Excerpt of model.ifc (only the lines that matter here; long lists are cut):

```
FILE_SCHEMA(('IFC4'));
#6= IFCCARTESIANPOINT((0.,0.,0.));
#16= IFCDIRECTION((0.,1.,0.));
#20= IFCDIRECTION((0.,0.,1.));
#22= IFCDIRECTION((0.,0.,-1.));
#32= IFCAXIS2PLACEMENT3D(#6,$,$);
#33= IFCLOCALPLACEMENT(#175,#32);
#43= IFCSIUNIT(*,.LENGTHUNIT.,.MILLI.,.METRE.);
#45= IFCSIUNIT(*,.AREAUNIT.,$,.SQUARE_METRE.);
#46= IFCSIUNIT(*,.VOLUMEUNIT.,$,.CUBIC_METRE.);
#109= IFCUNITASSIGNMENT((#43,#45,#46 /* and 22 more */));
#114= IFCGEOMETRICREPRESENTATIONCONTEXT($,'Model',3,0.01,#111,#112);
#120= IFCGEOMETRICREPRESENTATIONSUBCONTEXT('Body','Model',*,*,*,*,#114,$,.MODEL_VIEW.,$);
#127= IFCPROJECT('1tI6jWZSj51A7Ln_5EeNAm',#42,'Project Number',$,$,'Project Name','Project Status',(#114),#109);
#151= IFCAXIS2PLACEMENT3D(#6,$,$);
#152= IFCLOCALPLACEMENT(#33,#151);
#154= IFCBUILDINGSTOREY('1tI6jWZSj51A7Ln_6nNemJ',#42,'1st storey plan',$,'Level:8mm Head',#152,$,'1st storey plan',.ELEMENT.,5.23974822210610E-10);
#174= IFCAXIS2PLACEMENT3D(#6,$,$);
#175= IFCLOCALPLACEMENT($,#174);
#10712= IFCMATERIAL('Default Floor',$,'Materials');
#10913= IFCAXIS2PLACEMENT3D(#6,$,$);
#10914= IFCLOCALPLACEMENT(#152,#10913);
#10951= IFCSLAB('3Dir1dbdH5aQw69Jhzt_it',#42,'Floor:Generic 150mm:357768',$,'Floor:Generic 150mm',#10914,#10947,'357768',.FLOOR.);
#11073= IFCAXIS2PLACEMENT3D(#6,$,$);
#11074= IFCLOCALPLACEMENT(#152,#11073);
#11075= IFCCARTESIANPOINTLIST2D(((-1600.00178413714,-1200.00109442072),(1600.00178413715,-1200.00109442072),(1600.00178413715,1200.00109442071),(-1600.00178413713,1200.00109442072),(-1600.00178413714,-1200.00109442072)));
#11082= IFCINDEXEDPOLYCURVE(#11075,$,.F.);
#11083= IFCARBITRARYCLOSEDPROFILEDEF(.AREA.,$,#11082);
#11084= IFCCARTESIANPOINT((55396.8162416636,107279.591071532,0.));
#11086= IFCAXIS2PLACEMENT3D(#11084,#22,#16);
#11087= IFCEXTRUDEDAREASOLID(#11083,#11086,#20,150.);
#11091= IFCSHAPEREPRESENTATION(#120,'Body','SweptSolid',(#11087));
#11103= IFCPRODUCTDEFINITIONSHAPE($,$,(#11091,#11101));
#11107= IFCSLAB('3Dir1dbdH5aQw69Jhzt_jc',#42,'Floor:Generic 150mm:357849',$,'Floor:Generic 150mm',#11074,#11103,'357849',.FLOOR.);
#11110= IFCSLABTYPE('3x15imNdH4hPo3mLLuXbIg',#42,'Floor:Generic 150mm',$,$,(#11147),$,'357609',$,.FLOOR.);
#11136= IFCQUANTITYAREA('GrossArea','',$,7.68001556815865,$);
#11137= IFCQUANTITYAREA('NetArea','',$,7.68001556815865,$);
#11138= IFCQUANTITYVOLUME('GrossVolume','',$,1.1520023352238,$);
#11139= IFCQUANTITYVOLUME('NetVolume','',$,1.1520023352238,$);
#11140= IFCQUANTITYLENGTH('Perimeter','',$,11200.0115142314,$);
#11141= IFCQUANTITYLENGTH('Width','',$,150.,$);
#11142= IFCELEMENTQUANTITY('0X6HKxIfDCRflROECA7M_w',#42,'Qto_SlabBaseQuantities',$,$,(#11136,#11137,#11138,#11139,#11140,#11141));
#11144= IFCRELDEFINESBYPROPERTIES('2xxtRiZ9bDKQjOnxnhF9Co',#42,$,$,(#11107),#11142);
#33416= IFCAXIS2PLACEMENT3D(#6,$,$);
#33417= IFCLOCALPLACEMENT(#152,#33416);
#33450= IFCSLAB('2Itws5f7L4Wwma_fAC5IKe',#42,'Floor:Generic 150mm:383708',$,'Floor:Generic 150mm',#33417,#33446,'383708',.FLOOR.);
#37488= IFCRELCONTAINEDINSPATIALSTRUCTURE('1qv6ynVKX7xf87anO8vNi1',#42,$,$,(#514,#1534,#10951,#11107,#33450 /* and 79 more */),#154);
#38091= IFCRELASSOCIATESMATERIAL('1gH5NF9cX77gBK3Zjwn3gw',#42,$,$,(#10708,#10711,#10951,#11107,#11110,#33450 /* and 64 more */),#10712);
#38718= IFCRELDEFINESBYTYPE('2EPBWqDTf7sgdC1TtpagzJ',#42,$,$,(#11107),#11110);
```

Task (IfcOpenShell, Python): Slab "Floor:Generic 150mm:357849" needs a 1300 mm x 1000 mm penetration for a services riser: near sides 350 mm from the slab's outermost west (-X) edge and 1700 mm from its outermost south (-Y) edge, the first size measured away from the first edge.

```python
import numpy as np
import ifcopenshell
import ifcopenshell.api.feature
import ifcopenshell.api.geometry
import ifcopenshell.api.pset
import ifcopenshell.api.root
import ifcopenshell.geom
import ifcopenshell.util.element
import ifcopenshell.util.placement
import ifcopenshell.util.representation
import ifcopenshell.util.shape
import ifcopenshell.util.unit

model = ifcopenshell.open("model.ifc")
unit_scale = ifcopenshell.util.unit.calculate_unit_scale(model)
area_scale = ifcopenshell.util.unit.calculate_unit_scale(model, "AREAUNIT")
volume_scale = ifcopenshell.util.unit.calculate_unit_scale(model, "VOLUMEUNIT")
settings = ifcopenshell.geom.settings()


def volume(element):
    """Net volume in cubic metres, openings subtracted."""
    shape = ifcopenshell.geom.create_shape(settings, element)
    return ifcopenshell.util.shape.get_volume(shape.geometry)


slab = model.by_guid("3Dir1dbdH5aQw69Jhzt_jc")
before = volume(slab)

# Extent in the slab's own axes, in metres. The edges named are its -X and -Y sides.
slab_shape = ifcopenshell.geom.create_shape(settings, slab)
vertices = ifcopenshell.util.shape.get_vertices(slab_shape.geometry)
x_min, y_min, bottom = vertices.min(axis=0)
top = vertices[:, 2].max()

opening = ifcopenshell.api.root.create_entity(model, ifc_class="IfcOpeningElement", name="Services riser opening", predefined_type="OPENING")
context = ifcopenshell.util.representation.get_context(model, "Model", "Body", "MODEL_VIEW")
width, depth = 1.3, 1
outline = [(0.0, 0.0), (width, 0.0), (width, depth), (0.0, depth), (0.0, 0.0)]
# Overshoot both faces by 50 mm so the cut is clean.
shape = ifcopenshell.api.geometry.add_slab_representation(
    model, context=context, depth=top - bottom + 0.1, polyline=outline
)
ifcopenshell.api.geometry.assign_representation(model, product=opening, representation=shape)

matrix = ifcopenshell.util.placement.get_local_placement(slab.ObjectPlacement)
matrix[:, 3] = matrix @ np.append(np.array([x_min + 0.35, y_min + 1.7, bottom - 0.05]) / unit_scale, 1.0)
ifcopenshell.api.geometry.edit_object_placement(model, product=opening, matrix=matrix, is_si=False)
ifcopenshell.api.feature.add_feature(model, feature=opening, element=slab)

after = volume(slab)

# Update the slab's stored quantities.
qto = model.by_id(ifcopenshell.util.element.get_pset(slab, "Qto_SlabBaseQuantities", should_inherit=False)["id"])
ifcopenshell.api.pset.edit_qto(model, qto=qto, properties={
    "NetArea": after / (top - bottom) / area_scale,
    "NetVolume": after / volume_scale,
})

print(f"slab volume {before:.3f} -> {after:.3f} m3")

model.write("model_v2.ifc")
```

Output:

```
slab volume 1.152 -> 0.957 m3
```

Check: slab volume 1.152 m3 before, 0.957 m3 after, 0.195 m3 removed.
